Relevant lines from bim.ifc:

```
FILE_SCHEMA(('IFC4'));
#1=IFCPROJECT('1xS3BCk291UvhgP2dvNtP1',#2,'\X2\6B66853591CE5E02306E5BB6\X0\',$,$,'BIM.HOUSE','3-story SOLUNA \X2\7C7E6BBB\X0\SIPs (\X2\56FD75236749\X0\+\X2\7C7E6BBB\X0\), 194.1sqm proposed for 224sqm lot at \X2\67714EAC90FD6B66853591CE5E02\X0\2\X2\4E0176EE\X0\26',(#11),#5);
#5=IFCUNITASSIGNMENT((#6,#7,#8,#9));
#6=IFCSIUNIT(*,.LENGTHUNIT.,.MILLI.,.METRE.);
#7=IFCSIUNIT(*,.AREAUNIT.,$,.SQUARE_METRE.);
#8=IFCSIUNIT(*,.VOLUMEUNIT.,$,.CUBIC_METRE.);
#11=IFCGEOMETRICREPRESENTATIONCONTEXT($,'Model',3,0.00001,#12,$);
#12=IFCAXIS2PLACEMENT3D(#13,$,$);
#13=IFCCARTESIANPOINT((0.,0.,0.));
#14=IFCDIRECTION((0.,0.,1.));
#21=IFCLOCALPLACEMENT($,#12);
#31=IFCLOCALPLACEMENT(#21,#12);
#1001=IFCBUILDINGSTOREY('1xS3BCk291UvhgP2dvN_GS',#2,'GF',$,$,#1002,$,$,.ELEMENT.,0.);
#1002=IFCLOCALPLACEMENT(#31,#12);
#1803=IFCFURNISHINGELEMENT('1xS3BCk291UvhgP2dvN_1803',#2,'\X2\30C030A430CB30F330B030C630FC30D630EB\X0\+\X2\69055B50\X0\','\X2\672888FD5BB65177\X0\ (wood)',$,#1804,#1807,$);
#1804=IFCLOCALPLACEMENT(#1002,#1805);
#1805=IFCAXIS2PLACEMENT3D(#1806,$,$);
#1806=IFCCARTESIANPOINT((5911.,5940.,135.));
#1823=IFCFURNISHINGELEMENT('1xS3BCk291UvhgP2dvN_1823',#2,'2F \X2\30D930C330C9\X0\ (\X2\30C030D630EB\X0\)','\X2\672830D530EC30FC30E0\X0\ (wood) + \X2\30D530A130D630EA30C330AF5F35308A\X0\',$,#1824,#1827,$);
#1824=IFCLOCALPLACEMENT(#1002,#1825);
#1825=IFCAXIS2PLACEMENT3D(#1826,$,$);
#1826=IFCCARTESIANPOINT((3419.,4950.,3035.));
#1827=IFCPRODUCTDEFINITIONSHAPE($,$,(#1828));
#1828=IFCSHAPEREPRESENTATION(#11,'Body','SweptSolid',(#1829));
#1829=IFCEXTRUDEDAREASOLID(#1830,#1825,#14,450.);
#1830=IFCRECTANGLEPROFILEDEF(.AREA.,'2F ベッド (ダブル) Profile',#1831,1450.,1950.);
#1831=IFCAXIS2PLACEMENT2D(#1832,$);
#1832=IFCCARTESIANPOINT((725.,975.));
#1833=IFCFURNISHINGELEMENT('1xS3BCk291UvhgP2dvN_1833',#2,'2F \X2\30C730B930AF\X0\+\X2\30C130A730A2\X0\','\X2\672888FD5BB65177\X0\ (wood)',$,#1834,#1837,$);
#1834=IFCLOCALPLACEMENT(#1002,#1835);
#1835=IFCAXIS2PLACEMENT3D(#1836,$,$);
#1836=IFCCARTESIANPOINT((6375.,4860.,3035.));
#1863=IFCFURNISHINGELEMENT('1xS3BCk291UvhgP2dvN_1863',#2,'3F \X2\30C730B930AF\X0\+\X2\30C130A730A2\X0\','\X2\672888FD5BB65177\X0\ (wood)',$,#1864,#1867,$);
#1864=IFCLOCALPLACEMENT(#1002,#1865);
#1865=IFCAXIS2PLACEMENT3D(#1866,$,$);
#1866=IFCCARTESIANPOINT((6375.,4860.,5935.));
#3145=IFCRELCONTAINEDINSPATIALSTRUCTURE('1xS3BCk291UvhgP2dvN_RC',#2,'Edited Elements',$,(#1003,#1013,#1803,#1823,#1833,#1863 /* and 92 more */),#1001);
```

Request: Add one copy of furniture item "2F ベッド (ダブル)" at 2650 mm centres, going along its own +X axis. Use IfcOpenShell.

```python
import ifcopenshell
import ifcopenshell.api.geometry
import ifcopenshell.api.root
import ifcopenshell.util.element
import ifcopenshell.util.placement

model = ifcopenshell.open("bim.ifc")


def reuse_history(source, copy):
    """copy_class also copies each property set's owner history, people and application; keep the originals."""
    for rel in copy.IsDefinedBy:
        if rel.is_a("IfcRelDefinesByProperties") and (history := rel.RelatingPropertyDefinition.OwnerHistory):
            rel.RelatingPropertyDefinition.OwnerHistory = source.OwnerHistory
            ifcopenshell.util.element.remove_deep2(model, history)


source = model.by_guid("1xS3BCk291UvhgP2dvN_1823")
base = ifcopenshell.util.placement.get_local_placement(source.ObjectPlacement)
step = base[:3, 0] * 2650.0

for i in range(1, 2):
    copy = ifcopenshell.api.root.copy_class(model, product=source)
    copy.Representation = ifcopenshell.util.element.copy_deep(
        model, source.Representation, exclude=["IfcGeometricRepresentationContext", "IfcRepresentationMap"]
    )
    reuse_history(source, copy)
    matrix = base.copy()
    matrix[:3, 3] += i * step
    print("added at", matrix[:3, 3].round(3) + 0.0)
    ifcopenshell.api.geometry.edit_object_placement(model, product=copy, matrix=matrix, is_si=False)

model.write("bim_updated.ifc")
```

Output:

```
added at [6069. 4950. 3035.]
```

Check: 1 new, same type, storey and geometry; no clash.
